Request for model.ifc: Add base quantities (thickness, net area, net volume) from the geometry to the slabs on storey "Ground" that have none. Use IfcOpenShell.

First a look at what the model holds.

```python
import ifcopenshell
import ifcopenshell.util.element
import ifcopenshell.util.unit

model = ifcopenshell.open("model.ifc")
print(model.schema)
for unit_type in ("LENGTHUNIT", "AREAUNIT", "VOLUMEUNIT"):
    print(unit_type, ifcopenshell.util.unit.calculate_unit_scale(model, unit_type))
storey = next(s for s in model.by_type("IfcBuildingStorey") if s.Name == "Ground")
slabs = [e for e in ifcopenshell.util.element.get_decomposition(storey) if e.is_a("IfcSlab")]
for e in sorted(slabs, key=lambda e: e.id()):
    print(e.id(), e.is_a(), e.Name, list(ifcopenshell.util.element.get_psets(e, qtos_only=True)), sep=" | ")
```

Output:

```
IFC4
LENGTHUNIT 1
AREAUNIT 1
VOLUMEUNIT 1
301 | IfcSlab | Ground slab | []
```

```python
import ifcopenshell
import ifcopenshell.api.pset
import ifcopenshell.geom
import ifcopenshell.util.element
import ifcopenshell.util.shape
import ifcopenshell.util.unit

model = ifcopenshell.open("model.ifc")
unit_scale = ifcopenshell.util.unit.calculate_unit_scale(model)
area_scale = ifcopenshell.util.unit.calculate_unit_scale(model, "AREAUNIT")
volume_scale = ifcopenshell.util.unit.calculate_unit_scale(model, "VOLUMEUNIT")
settings = ifcopenshell.geom.settings()

storey = next(s for s in model.by_type("IfcBuildingStorey") if s.Name == "Ground")
slabs = [e for e in ifcopenshell.util.element.get_decomposition(storey) if e.is_a("IfcSlab")]

for e in sorted(slabs, key=lambda e: e.id()):
    if ifcopenshell.util.element.get_psets(e, qtos_only=True, should_inherit=False):
        continue
    # Geometry comes back in metres, in the element's own axes.
    shape = ifcopenshell.geom.create_shape(settings, e)
    values = {
        "Width": ifcopenshell.util.shape.get_z(shape.geometry) / unit_scale,
        "NetArea": ifcopenshell.util.shape.get_footprint_area(shape.geometry) / area_scale,
        "NetVolume": ifcopenshell.util.shape.get_volume(shape.geometry) / volume_scale,
    }
    qto = ifcopenshell.api.pset.add_qto(model, product=e, name="Qto_SlabBaseQuantities")
    ifcopenshell.api.pset.edit_qto(model, qto=qto, properties=values)
    print(e.id(), {k: round(v, 3) for k, v in values.items()})

model.write("model_updated.ifc")
```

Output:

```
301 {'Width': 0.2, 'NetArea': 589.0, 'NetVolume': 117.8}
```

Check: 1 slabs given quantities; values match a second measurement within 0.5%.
